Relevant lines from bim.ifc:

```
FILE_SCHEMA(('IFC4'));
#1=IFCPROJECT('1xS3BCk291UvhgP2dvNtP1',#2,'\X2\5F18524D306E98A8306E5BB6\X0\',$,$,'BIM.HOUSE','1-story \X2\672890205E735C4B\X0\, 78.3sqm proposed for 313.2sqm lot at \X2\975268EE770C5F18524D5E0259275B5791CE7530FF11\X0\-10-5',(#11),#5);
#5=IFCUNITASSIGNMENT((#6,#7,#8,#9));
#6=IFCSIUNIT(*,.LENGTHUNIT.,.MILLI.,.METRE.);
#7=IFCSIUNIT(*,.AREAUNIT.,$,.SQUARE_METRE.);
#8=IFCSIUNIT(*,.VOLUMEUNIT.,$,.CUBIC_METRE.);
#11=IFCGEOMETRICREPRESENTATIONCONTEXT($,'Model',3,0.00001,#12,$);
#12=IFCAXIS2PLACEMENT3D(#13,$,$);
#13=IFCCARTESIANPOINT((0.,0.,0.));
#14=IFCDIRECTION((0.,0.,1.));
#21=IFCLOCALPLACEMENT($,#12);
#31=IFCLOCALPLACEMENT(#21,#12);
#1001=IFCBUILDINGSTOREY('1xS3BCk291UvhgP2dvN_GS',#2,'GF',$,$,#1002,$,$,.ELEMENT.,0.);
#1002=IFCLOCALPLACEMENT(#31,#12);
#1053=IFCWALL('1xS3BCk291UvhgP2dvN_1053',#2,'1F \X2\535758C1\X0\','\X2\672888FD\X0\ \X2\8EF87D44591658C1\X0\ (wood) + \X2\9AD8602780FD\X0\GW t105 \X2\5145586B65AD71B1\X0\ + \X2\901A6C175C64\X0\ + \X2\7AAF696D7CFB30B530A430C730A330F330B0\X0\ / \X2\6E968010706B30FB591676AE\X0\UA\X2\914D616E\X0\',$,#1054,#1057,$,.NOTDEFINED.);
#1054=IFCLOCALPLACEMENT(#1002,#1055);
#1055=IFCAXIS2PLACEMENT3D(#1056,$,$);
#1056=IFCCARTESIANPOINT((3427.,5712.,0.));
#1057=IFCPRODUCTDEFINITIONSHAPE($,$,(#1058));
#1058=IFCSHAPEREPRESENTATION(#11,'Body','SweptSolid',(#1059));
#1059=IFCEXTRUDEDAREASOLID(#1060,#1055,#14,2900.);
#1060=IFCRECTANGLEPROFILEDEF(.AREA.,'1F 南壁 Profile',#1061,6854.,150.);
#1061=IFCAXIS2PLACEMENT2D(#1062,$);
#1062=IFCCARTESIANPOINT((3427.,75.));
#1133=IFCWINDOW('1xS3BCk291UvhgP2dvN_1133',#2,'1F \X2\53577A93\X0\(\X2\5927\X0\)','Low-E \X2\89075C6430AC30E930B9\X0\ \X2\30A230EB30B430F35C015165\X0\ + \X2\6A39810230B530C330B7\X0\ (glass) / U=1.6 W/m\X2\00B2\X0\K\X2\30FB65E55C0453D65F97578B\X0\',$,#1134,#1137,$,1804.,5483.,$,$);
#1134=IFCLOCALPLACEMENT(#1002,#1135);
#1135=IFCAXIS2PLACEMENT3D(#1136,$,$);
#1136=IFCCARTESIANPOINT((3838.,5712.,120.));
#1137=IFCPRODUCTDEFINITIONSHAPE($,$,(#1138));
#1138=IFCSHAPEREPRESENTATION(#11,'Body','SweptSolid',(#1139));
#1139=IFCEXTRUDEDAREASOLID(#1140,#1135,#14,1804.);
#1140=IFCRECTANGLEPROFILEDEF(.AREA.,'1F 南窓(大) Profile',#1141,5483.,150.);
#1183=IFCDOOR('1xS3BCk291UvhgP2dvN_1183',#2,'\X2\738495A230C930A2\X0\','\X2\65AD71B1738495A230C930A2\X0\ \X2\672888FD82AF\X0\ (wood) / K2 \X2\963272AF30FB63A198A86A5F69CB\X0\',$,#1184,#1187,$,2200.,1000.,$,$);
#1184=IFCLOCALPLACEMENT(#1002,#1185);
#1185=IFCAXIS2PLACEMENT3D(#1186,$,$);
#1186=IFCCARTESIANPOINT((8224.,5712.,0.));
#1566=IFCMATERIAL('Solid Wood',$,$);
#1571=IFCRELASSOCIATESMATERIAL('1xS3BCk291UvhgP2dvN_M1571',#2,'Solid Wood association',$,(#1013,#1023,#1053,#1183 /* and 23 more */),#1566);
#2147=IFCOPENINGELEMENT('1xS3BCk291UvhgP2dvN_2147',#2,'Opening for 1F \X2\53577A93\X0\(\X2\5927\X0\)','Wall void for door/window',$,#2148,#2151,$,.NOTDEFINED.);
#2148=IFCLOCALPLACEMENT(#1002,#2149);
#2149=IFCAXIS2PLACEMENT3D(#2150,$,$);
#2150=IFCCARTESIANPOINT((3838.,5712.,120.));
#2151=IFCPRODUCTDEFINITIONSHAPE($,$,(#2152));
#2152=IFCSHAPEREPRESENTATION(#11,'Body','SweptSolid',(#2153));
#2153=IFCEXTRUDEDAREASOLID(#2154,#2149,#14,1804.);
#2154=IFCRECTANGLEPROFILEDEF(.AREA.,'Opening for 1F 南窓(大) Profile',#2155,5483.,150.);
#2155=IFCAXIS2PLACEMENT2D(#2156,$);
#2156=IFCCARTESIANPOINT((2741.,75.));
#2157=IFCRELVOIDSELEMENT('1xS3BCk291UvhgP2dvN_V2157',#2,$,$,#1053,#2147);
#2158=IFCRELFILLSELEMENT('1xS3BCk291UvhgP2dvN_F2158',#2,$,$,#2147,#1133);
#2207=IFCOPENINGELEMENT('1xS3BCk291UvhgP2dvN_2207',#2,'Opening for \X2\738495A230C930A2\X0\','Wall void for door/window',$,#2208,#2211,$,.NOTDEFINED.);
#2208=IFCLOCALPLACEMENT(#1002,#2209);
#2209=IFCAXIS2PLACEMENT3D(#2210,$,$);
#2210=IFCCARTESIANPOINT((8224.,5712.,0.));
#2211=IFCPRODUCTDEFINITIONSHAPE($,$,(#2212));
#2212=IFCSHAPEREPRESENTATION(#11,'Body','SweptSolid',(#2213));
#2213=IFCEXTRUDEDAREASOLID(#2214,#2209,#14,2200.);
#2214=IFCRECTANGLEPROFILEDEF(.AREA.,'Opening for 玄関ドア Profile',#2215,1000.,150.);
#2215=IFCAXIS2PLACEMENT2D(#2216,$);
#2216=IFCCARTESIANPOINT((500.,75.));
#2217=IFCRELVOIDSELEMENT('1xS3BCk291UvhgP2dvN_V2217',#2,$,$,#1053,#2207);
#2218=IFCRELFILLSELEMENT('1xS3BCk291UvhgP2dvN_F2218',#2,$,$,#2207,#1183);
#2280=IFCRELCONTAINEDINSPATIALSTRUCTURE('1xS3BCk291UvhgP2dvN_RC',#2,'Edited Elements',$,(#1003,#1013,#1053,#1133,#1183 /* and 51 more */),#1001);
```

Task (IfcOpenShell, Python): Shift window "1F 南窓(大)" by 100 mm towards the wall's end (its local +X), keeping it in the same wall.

```python
import ifcopenshell
import ifcopenshell.api.geometry
import ifcopenshell.util.placement
import ifcopenshell.util.unit

model = ifcopenshell.open("bim.ifc")
unit_scale = ifcopenshell.util.unit.calculate_unit_scale(model)

window = model.by_guid("1xS3BCk291UvhgP2dvN_1133")
opening = window.FillsVoids[0].RelatingOpeningElement
wall = opening.VoidsElements[0].RelatingBuildingElement

wall_matrix = ifcopenshell.util.placement.get_local_placement(wall.ObjectPlacement)
shift = wall_matrix[:3, 0] * 0.1 / unit_scale
before = ifcopenshell.util.placement.get_local_placement(window.ObjectPlacement)[:3, 3].copy()

# The window is not placed relative to its opening, so move both.
for product in (opening, window):
    matrix = ifcopenshell.util.placement.get_local_placement(product.ObjectPlacement)
    matrix[:3, 3] += shift
    ifcopenshell.api.geometry.edit_object_placement(model, product=product, matrix=matrix, is_si=False)

after = ifcopenshell.util.placement.get_local_placement(window.ObjectPlacement)[:3, 3]
print("window moved by", (after - before).round(3) + 0.0)

model.write("bim_updated.ifc")
```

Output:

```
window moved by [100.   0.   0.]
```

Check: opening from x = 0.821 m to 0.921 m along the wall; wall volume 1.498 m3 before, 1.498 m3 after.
